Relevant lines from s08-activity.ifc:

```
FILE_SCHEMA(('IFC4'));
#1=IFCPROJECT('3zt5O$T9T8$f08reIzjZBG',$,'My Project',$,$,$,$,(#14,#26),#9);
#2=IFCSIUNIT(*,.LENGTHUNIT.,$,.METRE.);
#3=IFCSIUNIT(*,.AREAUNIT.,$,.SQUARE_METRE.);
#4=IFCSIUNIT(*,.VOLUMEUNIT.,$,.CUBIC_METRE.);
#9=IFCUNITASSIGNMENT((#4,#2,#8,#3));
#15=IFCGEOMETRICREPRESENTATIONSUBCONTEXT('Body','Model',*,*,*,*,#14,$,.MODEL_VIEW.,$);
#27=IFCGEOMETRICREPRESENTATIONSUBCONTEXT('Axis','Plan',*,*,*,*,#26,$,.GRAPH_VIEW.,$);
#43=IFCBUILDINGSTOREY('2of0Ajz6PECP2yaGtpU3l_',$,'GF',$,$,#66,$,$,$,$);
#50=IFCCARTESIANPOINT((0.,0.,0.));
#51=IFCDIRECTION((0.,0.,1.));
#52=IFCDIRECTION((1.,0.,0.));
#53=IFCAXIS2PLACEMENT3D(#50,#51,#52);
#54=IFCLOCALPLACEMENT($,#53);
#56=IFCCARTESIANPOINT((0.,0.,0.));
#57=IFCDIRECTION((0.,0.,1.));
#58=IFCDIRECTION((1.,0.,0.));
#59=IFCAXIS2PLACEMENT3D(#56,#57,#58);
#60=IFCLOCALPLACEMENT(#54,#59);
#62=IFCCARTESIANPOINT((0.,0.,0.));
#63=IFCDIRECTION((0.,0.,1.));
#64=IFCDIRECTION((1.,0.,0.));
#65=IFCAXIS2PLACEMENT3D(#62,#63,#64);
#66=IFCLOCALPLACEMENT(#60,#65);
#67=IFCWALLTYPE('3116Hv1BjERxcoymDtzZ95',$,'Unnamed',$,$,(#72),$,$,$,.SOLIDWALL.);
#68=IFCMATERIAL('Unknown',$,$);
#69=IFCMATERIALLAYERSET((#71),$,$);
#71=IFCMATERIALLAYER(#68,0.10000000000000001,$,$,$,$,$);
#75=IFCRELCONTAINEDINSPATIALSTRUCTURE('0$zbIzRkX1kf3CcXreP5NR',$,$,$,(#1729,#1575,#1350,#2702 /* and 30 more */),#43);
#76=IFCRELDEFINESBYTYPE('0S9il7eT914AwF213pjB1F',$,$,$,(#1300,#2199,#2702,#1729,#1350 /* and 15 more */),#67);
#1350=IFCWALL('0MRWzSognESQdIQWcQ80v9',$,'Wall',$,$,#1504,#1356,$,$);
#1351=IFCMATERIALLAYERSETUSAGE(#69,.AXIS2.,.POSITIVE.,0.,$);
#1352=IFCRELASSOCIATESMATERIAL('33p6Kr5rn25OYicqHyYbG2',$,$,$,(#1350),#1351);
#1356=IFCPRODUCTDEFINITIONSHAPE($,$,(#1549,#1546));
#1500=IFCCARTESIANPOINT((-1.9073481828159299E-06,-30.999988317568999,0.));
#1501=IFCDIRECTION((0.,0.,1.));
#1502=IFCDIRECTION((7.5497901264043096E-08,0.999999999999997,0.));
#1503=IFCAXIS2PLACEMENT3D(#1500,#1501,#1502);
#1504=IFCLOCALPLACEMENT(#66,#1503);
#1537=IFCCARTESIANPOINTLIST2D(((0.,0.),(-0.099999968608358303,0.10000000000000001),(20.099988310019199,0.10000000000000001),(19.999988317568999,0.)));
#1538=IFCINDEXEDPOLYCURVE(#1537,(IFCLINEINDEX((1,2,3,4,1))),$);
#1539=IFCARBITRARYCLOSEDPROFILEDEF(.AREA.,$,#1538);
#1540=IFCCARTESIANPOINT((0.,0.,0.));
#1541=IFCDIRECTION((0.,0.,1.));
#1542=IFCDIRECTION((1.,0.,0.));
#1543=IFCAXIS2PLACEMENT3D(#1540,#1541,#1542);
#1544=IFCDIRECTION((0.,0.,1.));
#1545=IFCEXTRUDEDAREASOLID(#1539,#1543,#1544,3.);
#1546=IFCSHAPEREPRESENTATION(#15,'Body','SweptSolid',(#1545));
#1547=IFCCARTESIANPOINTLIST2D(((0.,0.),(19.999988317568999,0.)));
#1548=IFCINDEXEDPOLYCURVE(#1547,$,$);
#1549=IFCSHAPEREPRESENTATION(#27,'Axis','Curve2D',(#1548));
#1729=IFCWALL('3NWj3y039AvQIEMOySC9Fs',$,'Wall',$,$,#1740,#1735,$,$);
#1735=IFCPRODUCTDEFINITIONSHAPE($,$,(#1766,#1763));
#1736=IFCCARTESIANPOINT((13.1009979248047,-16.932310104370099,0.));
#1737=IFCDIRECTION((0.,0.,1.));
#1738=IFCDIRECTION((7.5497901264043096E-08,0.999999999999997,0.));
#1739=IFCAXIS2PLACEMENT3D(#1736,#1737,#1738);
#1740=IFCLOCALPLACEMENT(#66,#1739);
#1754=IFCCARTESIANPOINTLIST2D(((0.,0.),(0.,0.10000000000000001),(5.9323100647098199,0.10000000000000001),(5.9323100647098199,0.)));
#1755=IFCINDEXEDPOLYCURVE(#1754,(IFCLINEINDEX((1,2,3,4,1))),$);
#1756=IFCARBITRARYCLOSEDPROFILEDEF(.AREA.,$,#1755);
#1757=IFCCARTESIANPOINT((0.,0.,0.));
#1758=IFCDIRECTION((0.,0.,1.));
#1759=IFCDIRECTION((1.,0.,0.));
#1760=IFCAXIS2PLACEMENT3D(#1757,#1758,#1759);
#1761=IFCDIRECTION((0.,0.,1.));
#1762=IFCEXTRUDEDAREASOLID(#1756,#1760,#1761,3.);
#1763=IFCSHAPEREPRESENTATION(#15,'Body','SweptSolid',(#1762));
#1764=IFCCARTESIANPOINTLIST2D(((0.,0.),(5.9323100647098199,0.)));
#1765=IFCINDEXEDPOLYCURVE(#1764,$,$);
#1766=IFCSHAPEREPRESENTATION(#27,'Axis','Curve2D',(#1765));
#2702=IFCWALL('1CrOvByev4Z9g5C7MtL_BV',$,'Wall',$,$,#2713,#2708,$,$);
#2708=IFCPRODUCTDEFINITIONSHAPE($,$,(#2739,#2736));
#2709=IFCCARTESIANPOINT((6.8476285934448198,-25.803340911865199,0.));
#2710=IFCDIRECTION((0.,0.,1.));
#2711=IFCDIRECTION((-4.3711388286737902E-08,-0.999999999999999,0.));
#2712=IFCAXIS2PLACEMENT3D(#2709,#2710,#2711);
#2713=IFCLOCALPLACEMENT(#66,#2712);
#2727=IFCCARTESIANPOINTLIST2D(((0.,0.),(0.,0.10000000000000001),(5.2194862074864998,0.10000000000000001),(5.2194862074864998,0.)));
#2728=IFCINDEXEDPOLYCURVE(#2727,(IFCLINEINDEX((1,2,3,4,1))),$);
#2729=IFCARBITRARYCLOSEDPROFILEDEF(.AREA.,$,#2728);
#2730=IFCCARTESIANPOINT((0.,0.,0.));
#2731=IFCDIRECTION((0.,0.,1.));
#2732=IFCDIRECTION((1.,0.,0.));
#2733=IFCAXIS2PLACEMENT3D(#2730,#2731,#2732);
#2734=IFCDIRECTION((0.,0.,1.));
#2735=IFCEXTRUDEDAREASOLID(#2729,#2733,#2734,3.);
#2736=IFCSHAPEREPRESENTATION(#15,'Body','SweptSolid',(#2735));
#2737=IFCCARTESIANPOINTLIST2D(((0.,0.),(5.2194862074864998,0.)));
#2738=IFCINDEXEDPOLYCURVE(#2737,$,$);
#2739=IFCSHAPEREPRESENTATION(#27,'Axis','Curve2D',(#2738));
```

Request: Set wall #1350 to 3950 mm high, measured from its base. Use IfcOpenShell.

```python
import ifcopenshell
import ifcopenshell.geom
import ifcopenshell.util.representation
import ifcopenshell.util.shape
import ifcopenshell.util.unit

model = ifcopenshell.open("s08-activity.ifc")
unit_scale = ifcopenshell.util.unit.calculate_unit_scale(model)
settings = ifcopenshell.geom.settings()


def volume(element):
    """Net volume in cubic metres, openings subtracted."""
    shape = ifcopenshell.geom.create_shape(settings, element)
    return ifcopenshell.util.shape.get_volume(shape.geometry)


wall = model.by_guid("0MRWzSognESQdIQWcQ80v9")
before = volume(wall)

body = ifcopenshell.util.representation.get_representation(wall, "Model", "Body")
solid = body.Items[0]
old_height = solid.Depth
solid.Depth = 3.95 / unit_scale
after = volume(wall)

print(f"height {old_height:g} -> {solid.Depth:g}, volume {before:.3f} -> {after:.3f} m3")

model.write("s08-activity_edited.ifc")
```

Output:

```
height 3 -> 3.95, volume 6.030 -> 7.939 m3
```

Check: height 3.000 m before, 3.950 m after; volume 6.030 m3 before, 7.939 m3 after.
